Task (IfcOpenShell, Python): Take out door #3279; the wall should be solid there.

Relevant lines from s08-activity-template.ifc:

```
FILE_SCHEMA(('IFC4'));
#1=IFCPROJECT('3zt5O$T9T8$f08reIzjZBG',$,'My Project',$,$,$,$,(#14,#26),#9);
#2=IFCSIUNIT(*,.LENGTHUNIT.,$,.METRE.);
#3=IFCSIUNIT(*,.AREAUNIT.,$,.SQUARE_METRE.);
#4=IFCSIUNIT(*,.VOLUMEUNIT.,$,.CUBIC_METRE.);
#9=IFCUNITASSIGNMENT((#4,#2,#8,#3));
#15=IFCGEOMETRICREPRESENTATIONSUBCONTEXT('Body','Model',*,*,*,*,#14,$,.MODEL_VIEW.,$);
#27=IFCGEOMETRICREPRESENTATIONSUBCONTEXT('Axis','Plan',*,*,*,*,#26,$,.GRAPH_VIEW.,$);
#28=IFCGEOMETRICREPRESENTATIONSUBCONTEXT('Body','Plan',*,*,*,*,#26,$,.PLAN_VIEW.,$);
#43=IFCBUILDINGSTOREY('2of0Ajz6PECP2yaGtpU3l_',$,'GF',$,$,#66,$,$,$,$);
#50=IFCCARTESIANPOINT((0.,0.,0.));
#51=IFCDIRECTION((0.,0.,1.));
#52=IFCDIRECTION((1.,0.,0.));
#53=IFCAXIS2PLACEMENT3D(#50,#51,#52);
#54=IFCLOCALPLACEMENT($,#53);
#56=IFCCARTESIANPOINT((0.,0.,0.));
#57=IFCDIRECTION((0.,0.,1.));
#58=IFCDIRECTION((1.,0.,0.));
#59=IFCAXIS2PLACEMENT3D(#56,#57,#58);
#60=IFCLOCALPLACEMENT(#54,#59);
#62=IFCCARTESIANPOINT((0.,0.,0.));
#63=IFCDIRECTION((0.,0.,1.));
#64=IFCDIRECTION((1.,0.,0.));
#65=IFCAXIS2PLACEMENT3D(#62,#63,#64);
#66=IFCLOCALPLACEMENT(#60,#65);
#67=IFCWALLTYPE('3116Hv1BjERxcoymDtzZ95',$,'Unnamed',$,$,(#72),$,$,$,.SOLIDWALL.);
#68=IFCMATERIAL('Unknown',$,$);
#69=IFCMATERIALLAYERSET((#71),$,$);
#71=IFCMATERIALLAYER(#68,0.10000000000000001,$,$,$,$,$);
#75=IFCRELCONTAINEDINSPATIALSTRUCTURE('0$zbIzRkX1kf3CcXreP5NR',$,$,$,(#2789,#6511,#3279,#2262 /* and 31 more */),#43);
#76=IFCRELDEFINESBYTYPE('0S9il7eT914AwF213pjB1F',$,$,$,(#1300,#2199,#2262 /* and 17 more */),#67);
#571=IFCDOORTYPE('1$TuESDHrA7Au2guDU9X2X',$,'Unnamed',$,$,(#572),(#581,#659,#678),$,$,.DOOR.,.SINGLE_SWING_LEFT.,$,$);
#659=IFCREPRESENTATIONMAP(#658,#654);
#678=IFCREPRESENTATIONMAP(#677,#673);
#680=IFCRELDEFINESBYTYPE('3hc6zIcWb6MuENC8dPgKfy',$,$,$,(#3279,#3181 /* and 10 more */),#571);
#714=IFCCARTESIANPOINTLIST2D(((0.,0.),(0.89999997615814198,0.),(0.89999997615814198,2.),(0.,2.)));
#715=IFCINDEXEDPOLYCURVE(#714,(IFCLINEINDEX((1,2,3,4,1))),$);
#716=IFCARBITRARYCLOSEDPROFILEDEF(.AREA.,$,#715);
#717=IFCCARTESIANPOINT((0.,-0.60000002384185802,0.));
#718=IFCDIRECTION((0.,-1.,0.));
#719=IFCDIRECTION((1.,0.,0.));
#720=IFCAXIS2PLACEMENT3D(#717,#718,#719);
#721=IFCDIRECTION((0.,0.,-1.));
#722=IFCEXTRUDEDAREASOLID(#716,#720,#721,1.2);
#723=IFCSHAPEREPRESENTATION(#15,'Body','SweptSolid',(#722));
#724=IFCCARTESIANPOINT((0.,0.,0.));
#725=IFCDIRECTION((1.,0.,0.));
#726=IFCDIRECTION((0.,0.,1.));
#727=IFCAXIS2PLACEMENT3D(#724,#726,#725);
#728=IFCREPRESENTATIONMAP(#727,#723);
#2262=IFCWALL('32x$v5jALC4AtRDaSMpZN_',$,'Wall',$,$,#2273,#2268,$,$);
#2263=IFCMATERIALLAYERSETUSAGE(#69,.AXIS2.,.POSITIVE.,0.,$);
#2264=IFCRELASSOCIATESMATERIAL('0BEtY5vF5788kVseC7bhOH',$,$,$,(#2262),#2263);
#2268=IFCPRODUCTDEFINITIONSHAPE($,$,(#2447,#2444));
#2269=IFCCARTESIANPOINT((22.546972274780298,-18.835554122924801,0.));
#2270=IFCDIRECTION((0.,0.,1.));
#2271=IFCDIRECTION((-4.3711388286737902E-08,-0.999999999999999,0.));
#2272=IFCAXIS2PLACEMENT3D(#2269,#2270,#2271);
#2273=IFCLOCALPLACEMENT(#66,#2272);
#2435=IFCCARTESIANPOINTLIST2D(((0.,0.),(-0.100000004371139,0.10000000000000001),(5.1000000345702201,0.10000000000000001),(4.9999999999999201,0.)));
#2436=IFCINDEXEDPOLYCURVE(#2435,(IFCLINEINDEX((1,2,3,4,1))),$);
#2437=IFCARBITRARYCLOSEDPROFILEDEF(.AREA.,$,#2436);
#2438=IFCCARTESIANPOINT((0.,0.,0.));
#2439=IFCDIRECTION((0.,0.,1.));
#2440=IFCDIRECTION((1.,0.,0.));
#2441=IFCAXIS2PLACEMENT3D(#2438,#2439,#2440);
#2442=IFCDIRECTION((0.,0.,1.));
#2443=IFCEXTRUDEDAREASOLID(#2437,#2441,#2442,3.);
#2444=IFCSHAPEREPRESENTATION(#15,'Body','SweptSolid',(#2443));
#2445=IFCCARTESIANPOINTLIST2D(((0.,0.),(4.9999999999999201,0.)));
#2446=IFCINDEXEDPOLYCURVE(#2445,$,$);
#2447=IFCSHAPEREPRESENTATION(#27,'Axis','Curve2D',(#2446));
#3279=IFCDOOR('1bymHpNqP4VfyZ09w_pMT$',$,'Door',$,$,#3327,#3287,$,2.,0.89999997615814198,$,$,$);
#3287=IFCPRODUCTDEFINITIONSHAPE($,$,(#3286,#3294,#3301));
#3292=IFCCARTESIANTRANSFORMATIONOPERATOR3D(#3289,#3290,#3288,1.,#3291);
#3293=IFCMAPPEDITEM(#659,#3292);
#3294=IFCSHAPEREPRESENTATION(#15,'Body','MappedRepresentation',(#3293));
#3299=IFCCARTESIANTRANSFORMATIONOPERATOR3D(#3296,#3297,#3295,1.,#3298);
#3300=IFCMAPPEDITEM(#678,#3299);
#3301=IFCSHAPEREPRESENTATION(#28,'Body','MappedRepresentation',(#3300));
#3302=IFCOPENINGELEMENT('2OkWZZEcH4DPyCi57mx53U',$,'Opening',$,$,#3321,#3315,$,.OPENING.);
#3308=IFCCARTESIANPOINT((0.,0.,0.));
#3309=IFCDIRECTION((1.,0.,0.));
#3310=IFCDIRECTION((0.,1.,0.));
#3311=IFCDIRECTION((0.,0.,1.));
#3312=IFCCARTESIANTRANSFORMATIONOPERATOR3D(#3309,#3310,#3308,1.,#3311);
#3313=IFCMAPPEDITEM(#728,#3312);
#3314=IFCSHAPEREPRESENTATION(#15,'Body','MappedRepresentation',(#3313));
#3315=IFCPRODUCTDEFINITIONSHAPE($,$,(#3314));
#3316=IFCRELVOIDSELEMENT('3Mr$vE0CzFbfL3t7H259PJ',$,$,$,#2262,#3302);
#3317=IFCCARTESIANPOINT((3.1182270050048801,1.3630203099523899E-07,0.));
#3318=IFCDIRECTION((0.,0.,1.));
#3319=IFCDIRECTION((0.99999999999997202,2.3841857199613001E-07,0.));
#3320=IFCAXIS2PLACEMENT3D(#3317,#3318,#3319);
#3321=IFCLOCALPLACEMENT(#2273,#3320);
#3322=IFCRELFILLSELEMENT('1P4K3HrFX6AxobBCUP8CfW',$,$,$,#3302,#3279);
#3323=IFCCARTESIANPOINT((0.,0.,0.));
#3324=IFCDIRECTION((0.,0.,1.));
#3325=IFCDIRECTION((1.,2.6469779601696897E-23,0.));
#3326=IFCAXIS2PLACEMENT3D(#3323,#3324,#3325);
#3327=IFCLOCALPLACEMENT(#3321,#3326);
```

```python
import ifcopenshell
import ifcopenshell.api.feature
import ifcopenshell.api.root
import ifcopenshell.geom
import ifcopenshell.util.shape

model = ifcopenshell.open("s08-activity-template.ifc")
settings = ifcopenshell.geom.settings()


def volume(element):
    """Net volume in cubic metres, openings subtracted."""
    shape = ifcopenshell.geom.create_shape(settings, element)
    return ifcopenshell.util.shape.get_volume(shape.geometry)


door = model.by_id(3279)
opening = door.FillsVoids[0].RelatingOpeningElement
wall = opening.VoidsElements[0].RelatingBuildingElement
before = volume(wall)

ifcopenshell.api.root.remove_product(model, product=door)
ifcopenshell.api.feature.remove_feature(model, feature=opening)

after = volume(wall)

print(f"wall volume {before:.3f} -> {after:.3f} m3")

model.write("s08-activity-template-out.ifc")
```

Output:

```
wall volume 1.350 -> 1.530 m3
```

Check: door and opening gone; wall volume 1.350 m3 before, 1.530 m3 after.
